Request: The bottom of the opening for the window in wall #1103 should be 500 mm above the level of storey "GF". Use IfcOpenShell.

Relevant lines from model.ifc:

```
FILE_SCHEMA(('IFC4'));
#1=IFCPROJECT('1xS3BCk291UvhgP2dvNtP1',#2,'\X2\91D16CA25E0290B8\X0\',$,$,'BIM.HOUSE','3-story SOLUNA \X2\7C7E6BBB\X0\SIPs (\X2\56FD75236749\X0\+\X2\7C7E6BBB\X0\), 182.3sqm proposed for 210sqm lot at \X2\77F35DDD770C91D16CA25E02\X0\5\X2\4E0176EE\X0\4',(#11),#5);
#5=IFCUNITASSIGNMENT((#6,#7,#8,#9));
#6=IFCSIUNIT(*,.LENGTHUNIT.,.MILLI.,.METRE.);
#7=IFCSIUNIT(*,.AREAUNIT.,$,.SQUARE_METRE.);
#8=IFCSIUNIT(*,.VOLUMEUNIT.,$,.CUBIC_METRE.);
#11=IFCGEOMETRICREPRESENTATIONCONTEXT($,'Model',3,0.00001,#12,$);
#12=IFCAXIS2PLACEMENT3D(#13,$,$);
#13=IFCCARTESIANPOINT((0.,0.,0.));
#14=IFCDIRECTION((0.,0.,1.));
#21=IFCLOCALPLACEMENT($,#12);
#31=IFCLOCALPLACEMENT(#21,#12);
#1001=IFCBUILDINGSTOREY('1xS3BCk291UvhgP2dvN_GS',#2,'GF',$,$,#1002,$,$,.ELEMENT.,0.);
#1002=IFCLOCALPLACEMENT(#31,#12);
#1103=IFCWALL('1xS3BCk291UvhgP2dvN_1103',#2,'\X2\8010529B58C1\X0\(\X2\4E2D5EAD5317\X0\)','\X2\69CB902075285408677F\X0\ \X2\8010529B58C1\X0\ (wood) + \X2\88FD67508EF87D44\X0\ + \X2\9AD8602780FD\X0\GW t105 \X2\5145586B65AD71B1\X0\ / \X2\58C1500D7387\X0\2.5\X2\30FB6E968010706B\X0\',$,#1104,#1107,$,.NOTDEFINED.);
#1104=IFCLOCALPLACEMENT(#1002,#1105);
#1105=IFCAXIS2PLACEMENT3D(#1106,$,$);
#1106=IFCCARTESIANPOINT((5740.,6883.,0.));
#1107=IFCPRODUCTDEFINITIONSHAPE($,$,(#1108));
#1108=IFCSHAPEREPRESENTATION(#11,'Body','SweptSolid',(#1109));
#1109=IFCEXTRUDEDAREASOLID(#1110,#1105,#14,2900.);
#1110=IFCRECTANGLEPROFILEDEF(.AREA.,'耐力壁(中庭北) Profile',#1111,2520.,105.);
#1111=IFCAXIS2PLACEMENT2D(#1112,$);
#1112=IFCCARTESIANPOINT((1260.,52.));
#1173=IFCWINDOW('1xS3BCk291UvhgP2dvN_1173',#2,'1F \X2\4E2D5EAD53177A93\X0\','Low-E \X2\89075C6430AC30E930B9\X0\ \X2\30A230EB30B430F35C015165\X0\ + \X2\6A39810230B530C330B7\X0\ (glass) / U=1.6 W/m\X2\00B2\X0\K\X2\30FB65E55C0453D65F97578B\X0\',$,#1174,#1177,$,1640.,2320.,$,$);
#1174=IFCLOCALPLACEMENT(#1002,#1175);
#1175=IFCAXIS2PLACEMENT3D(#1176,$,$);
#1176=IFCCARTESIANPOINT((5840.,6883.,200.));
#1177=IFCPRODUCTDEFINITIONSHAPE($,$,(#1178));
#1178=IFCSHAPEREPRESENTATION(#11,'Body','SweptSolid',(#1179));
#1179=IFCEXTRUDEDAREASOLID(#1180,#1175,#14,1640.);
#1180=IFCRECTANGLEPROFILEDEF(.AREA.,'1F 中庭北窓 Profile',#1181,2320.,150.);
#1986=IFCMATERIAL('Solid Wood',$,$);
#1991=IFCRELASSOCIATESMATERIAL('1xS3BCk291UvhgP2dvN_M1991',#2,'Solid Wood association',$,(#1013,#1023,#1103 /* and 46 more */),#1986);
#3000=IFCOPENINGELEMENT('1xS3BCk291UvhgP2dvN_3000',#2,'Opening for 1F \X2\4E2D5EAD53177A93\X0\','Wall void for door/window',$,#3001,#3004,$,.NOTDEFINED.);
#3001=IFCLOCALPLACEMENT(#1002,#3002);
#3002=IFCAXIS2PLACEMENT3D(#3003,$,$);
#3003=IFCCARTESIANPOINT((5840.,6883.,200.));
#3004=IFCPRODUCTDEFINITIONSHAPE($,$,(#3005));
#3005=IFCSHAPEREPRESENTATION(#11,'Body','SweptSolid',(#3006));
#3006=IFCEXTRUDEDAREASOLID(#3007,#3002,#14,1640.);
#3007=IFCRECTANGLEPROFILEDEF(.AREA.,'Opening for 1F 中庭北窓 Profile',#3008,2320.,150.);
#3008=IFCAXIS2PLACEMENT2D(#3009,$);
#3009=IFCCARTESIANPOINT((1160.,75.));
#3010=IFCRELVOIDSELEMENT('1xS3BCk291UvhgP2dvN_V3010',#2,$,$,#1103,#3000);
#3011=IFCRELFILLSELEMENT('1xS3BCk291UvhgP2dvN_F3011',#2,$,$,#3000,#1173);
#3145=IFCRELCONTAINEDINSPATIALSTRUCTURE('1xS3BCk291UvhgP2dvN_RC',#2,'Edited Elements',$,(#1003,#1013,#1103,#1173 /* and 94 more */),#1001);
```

```python
import numpy as np
import ifcopenshell
import ifcopenshell.api.geometry
import ifcopenshell.geom
import ifcopenshell.util.element
import ifcopenshell.util.placement
import ifcopenshell.util.shape
import ifcopenshell.util.unit

model = ifcopenshell.open("model.ifc")
unit_scale = ifcopenshell.util.unit.calculate_unit_scale(model)

window = model.by_guid("1xS3BCk291UvhgP2dvN_1173")
opening = window.FillsVoids[0].RelatingOpeningElement
storey = ifcopenshell.util.element.get_container(window, ifc_class="IfcBuildingStorey")
level = ifcopenshell.util.placement.get_local_placement(storey.ObjectPlacement)[2, 3]

# The opening's origin need not be at the sill, so measure its lowest point.
shape = ifcopenshell.geom.create_shape(ifcopenshell.geom.settings(), opening)
bottom = ifcopenshell.util.shape.get_shape_bottom_elevation(shape, shape.geometry) / unit_scale
dz = level + 500.0 - bottom

shift = np.array([0.0, 0.0, dz])
# The window is not placed relative to its opening, so move both.
for product in (opening, window):
    matrix = ifcopenshell.util.placement.get_local_placement(product.ObjectPlacement)
    matrix[:3, 3] += shift
    ifcopenshell.api.geometry.edit_object_placement(model, product=product, matrix=matrix, is_si=False)

print(f"moved by {dz * unit_scale:+.3f} m")

model.write("model-out.ifc")
```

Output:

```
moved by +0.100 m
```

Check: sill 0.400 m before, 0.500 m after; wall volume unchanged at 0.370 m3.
